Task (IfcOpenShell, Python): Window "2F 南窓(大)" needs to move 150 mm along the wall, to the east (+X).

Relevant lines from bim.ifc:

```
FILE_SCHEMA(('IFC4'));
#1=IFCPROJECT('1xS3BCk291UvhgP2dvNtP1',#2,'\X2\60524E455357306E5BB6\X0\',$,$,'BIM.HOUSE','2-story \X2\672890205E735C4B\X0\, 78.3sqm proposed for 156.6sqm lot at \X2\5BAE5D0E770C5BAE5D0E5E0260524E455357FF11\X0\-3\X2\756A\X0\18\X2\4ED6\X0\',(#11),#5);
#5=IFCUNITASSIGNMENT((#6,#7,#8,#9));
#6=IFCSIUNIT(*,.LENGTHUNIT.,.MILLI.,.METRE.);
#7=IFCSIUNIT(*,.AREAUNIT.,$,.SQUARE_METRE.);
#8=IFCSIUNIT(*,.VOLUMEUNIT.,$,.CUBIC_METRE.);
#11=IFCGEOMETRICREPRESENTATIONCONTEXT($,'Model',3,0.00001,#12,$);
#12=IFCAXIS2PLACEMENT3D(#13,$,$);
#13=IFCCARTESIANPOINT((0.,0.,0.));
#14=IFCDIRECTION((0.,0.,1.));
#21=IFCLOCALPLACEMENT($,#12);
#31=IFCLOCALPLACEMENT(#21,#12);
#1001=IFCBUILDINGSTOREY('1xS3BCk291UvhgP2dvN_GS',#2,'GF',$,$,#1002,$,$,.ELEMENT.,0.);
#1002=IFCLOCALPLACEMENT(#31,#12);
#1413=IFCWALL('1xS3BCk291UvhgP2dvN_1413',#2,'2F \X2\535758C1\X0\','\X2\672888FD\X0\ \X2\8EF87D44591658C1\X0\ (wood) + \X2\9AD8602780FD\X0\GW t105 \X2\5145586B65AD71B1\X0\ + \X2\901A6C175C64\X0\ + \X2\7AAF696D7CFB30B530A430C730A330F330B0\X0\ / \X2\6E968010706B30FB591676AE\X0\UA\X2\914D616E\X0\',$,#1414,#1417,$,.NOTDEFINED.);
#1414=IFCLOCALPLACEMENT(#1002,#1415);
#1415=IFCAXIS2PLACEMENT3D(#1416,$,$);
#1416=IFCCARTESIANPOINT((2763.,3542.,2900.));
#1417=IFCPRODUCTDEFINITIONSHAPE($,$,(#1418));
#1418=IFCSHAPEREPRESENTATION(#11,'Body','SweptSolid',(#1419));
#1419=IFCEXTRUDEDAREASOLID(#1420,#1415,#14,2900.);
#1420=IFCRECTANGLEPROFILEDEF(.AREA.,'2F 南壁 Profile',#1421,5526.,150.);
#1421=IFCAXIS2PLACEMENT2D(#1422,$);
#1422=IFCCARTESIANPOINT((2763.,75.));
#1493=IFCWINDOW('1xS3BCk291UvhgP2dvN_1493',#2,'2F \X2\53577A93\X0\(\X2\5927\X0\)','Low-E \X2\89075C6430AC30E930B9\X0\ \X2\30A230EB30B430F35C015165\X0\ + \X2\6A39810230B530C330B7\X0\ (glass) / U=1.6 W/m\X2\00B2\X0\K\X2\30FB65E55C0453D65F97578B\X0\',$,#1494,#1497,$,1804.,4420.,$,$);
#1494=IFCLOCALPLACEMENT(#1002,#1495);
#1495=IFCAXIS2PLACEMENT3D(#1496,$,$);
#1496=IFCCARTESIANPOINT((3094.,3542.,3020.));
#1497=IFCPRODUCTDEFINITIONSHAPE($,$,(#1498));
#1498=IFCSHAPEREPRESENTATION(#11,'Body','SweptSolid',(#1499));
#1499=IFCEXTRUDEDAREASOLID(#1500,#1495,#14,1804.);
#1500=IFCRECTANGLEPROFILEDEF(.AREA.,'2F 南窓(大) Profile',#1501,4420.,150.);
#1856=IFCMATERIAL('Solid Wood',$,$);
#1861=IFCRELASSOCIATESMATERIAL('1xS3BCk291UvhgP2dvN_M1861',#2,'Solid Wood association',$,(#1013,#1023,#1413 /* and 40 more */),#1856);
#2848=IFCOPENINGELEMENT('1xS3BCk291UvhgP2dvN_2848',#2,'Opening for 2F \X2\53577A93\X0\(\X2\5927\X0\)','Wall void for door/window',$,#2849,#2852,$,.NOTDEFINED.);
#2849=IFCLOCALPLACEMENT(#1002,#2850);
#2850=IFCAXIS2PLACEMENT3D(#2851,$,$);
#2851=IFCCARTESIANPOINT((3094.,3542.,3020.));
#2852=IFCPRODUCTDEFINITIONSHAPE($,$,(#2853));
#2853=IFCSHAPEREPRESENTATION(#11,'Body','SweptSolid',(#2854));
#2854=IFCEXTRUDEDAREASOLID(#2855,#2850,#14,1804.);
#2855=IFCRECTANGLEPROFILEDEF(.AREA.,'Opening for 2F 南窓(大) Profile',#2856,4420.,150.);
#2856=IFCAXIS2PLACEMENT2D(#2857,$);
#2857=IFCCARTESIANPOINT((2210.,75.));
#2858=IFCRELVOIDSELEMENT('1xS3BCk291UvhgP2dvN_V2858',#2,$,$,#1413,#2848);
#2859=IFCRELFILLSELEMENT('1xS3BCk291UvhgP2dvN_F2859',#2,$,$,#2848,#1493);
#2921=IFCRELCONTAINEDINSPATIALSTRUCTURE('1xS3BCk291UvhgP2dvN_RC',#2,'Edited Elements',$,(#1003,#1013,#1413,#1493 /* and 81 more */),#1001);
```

```python
import ifcopenshell
import ifcopenshell.api.geometry
import ifcopenshell.util.placement

model = ifcopenshell.open("bim.ifc")

window = model.by_guid("1xS3BCk291UvhgP2dvN_1493")
opening = window.FillsVoids[0].RelatingOpeningElement
wall = opening.VoidsElements[0].RelatingBuildingElement

wall_matrix = ifcopenshell.util.placement.get_local_placement(wall.ObjectPlacement)
shift = wall_matrix[:3, 0] * 150.0
before = ifcopenshell.util.placement.get_local_placement(window.ObjectPlacement)[:3, 3].copy()

# The window is not placed relative to its opening, so move both.
for product in (opening, window):
    matrix = ifcopenshell.util.placement.get_local_placement(product.ObjectPlacement)
    matrix[:3, 3] += shift
    ifcopenshell.api.geometry.edit_object_placement(model, product=product, matrix=matrix, is_si=False)

after = ifcopenshell.util.placement.get_local_placement(window.ObjectPlacement)[:3, 3]
print("window moved by", (after - before).round(3) + 0.0)

model.write("bim_updated.ifc")
```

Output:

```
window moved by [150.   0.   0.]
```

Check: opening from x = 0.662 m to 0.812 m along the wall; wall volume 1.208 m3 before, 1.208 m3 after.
